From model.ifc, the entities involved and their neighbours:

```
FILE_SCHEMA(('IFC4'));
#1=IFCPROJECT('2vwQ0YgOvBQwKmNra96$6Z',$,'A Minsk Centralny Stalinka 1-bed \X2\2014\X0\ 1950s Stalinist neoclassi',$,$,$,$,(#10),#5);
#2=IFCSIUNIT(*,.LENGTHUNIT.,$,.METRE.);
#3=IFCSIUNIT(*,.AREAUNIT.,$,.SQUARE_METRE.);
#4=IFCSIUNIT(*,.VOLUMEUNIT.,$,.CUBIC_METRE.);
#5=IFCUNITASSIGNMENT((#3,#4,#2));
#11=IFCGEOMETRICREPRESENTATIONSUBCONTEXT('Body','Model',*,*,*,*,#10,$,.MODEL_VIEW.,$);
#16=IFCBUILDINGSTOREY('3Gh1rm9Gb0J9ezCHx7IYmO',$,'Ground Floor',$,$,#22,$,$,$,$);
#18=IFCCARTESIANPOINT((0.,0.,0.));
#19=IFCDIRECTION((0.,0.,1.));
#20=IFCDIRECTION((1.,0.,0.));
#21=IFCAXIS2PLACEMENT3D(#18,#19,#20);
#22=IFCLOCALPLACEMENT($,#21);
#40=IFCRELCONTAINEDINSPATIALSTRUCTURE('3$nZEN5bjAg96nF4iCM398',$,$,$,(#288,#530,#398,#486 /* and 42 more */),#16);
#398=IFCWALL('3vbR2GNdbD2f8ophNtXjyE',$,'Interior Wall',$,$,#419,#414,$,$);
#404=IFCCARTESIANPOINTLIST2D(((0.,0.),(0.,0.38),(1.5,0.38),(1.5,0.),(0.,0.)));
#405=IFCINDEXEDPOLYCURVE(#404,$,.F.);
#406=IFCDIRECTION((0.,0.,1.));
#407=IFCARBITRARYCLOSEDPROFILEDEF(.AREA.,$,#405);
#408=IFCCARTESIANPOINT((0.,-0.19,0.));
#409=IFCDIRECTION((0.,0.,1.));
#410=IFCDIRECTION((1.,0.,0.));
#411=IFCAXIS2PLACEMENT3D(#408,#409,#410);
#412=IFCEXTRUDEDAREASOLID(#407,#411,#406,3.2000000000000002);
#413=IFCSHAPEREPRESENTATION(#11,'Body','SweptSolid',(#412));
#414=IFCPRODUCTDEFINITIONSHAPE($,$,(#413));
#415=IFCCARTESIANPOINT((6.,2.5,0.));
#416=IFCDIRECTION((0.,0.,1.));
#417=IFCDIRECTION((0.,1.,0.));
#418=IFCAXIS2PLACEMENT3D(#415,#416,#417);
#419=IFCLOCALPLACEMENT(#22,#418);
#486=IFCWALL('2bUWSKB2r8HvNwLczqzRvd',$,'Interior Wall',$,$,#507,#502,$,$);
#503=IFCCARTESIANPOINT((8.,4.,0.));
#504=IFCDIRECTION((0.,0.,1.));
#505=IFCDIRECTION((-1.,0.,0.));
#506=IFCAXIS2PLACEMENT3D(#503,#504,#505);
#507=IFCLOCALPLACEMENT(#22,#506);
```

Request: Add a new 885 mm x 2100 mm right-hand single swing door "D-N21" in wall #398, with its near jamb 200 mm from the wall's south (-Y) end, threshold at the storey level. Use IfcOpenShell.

```python
import numpy as np
import ifcopenshell
import ifcopenshell.api.feature
import ifcopenshell.api.geometry
import ifcopenshell.api.root
import ifcopenshell.api.spatial
import ifcopenshell.geom
import ifcopenshell.util.element
import ifcopenshell.util.placement
import ifcopenshell.util.representation
import ifcopenshell.util.shape
import ifcopenshell.util.unit

model = ifcopenshell.open("model.ifc")
unit_scale = ifcopenshell.util.unit.calculate_unit_scale(model)
settings = ifcopenshell.geom.settings()


def volume(element):
    """Net volume in cubic metres, openings subtracted."""
    shape = ifcopenshell.geom.create_shape(settings, element)
    return ifcopenshell.util.shape.get_volume(shape.geometry)


wall = model.by_id(398)
storey = ifcopenshell.util.element.get_container(wall, ifc_class="IfcBuildingStorey")
context = ifcopenshell.util.representation.get_context(model, "Model", "Body", "MODEL_VIEW")
before = volume(wall)

width, height, from_end, sill = 0.885, 2.1, 0.2, 0.0  # metres

# The wall runs along its own X axis, and the end named is its -X end.
wall_shape = ifcopenshell.geom.create_shape(settings, wall)
x, y, z = ifcopenshell.util.shape.get_vertices(wall_shape.geometry).T
start = x.min() + from_end
face, thickness = float(y.min()), float(y.max() - y.min())
wall_matrix = ifcopenshell.util.placement.get_local_placement(wall.ObjectPlacement)
level = ifcopenshell.util.placement.get_local_placement(storey.ObjectPlacement)[2, 3]


def in_wall(x, y):
    """Placement at x, y metres in the wall's axes, at sill height."""
    matrix = wall_matrix.copy()
    matrix[:, 3] = wall_matrix @ np.array([x / unit_scale, y / unit_scale, 0.0, 1.0])
    matrix[2, 3] = level + sill / unit_scale
    return matrix


# Opening: a box that overshoots both wall faces by 50 mm.
opening = ifcopenshell.api.root.create_entity(model, ifc_class="IfcOpeningElement", predefined_type="OPENING")
box = ifcopenshell.api.geometry.add_wall_representation(
    model, context=context, length=width, height=height, thickness=thickness + 0.1
)
ifcopenshell.api.geometry.assign_representation(model, product=opening, representation=box)
ifcopenshell.api.geometry.edit_object_placement(model, product=opening, matrix=in_wall(start, face - 0.05), is_si=False)
ifcopenshell.api.feature.add_feature(model, feature=opening, element=wall)

door = ifcopenshell.api.root.create_entity(model, ifc_class="IfcDoor", name="D-N21", predefined_type="DOOR")
door.OverallWidth, door.OverallHeight = width / unit_scale, height / unit_scale
door.OperationType = "SINGLE_SWING_RIGHT"
body = ifcopenshell.api.geometry.add_door_representation(
    model,
    context=context,
    overall_width=door.OverallWidth,
    overall_height=door.OverallHeight,
    operation_type="SINGLE_SWING_RIGHT",
    lining_properties={"LiningDepth": thickness / unit_scale, "ThresholdDepth": thickness / unit_scale},
)
ifcopenshell.api.geometry.assign_representation(model, product=door, representation=body)
ifcopenshell.api.spatial.assign_container(model, products=[door], relating_structure=storey)
ifcopenshell.api.feature.add_filling(model, opening=opening, element=door)

# The lining spans the wall, so the door starts at the wall face.
ifcopenshell.api.geometry.edit_object_placement(model, product=door, matrix=in_wall(start, face), is_si=False)

after = volume(wall)

print(f"wall volume {before:.3f} -> {after:.3f} m3")

model.write("model_rev.ifc")
```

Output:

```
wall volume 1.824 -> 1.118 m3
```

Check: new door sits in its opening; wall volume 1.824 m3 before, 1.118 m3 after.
